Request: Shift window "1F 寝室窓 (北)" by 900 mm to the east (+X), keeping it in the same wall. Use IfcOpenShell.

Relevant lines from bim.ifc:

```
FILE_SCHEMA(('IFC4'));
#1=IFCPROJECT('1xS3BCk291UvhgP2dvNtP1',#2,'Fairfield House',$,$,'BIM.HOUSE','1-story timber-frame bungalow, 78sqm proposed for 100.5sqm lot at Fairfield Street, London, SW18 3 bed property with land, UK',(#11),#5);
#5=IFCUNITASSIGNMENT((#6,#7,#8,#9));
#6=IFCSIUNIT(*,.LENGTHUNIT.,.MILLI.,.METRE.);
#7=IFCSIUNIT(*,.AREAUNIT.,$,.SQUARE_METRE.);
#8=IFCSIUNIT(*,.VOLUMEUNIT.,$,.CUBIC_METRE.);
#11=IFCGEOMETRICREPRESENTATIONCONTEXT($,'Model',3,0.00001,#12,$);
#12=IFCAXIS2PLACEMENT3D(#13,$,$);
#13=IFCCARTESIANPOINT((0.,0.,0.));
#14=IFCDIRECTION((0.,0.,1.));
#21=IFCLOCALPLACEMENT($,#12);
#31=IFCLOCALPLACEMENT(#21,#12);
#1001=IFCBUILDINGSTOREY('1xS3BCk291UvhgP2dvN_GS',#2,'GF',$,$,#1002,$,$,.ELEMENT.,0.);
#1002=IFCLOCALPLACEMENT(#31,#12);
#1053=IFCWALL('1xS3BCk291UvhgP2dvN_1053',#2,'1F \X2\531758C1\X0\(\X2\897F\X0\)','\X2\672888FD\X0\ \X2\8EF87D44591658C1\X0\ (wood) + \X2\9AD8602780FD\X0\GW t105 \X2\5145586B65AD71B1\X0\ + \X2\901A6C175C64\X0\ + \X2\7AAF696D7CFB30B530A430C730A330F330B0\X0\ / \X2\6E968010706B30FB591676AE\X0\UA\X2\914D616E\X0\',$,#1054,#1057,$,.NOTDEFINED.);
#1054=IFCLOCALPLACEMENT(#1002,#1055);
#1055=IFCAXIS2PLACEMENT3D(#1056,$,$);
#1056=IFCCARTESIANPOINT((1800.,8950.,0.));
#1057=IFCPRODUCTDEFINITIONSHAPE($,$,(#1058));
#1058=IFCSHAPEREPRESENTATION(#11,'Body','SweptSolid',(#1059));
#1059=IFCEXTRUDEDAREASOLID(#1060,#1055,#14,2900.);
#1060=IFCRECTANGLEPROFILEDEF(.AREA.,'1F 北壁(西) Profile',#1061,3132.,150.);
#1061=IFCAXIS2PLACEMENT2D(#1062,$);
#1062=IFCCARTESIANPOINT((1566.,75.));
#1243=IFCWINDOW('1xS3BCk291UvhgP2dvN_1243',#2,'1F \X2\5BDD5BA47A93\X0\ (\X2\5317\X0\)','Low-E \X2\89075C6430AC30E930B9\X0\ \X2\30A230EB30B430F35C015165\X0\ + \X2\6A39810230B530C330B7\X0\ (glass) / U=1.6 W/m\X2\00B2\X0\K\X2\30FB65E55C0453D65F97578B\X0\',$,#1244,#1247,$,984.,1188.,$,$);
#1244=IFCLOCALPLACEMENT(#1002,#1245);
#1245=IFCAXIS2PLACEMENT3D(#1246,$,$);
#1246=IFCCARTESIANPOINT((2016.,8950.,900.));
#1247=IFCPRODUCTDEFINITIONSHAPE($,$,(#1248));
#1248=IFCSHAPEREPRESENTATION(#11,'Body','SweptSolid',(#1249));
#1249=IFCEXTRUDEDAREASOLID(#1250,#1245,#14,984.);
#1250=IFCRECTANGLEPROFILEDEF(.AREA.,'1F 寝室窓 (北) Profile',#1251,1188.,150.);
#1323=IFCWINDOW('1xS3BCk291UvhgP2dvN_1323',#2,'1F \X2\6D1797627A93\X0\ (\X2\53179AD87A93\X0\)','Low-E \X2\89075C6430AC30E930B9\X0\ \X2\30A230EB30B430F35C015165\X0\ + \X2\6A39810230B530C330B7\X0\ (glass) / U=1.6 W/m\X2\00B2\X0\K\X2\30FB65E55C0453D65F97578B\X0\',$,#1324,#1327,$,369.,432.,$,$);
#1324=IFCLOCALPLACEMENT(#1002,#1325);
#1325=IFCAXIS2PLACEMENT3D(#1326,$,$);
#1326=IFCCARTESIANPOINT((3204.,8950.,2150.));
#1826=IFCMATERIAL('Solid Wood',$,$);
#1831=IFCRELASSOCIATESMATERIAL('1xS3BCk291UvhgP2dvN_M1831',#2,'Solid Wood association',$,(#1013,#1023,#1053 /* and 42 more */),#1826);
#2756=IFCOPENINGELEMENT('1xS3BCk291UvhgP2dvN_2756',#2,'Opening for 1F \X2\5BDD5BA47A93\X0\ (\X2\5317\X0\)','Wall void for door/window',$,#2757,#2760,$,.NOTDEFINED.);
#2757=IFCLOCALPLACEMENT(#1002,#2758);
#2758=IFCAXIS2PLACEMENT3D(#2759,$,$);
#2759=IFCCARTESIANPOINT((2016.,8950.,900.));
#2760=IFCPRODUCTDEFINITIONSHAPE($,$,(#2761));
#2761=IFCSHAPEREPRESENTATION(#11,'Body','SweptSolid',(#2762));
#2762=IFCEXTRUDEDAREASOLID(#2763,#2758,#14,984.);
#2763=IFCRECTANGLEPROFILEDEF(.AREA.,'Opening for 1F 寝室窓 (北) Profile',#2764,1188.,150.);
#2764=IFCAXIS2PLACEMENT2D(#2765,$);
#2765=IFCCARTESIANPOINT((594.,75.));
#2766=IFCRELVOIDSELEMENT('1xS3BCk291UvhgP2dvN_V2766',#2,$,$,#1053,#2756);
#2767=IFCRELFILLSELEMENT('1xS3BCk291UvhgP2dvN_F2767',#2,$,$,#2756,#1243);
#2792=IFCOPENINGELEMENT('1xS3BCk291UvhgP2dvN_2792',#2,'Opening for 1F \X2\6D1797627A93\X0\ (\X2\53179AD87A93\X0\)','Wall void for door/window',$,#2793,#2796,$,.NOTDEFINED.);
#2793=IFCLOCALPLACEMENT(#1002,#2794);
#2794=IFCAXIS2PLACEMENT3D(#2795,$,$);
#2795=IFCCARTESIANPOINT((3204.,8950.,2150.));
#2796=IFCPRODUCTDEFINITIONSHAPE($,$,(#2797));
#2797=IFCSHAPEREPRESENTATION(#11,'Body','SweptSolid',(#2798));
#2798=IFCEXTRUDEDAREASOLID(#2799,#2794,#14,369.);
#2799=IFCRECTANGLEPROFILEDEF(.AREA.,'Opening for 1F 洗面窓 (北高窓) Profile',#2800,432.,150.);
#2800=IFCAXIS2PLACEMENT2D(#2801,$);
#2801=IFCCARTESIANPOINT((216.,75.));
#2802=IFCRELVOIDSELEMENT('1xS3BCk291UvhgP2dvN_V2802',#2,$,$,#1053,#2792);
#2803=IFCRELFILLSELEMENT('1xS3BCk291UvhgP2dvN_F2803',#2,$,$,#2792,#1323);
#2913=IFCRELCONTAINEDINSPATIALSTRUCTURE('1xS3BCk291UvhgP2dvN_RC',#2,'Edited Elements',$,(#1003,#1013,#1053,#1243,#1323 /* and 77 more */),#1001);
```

```python
import ifcopenshell
import ifcopenshell.api.geometry
import ifcopenshell.util.placement
import ifcopenshell.util.unit

model = ifcopenshell.open("bim.ifc")
unit_scale = ifcopenshell.util.unit.calculate_unit_scale(model)

window = model.by_guid("1xS3BCk291UvhgP2dvN_1243")
opening = window.FillsVoids[0].RelatingOpeningElement
wall = opening.VoidsElements[0].RelatingBuildingElement

wall_matrix = ifcopenshell.util.placement.get_local_placement(wall.ObjectPlacement)
shift = wall_matrix[:3, 0] * 0.9 / unit_scale
before = ifcopenshell.util.placement.get_local_placement(window.ObjectPlacement)[:3, 3].copy()

# The window is not placed relative to its opening, so move both.
for product in (opening, window):
    matrix = ifcopenshell.util.placement.get_local_placement(product.ObjectPlacement)
    matrix[:3, 3] += shift
    ifcopenshell.api.geometry.edit_object_placement(model, product=product, matrix=matrix, is_si=False)

after = ifcopenshell.util.placement.get_local_placement(window.ObjectPlacement)[:3, 3]
print("window moved by", (after - before).round(3) + 0.0)

model.write("bim_updated.ifc")
```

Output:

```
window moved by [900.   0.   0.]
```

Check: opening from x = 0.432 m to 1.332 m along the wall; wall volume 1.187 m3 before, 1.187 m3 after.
